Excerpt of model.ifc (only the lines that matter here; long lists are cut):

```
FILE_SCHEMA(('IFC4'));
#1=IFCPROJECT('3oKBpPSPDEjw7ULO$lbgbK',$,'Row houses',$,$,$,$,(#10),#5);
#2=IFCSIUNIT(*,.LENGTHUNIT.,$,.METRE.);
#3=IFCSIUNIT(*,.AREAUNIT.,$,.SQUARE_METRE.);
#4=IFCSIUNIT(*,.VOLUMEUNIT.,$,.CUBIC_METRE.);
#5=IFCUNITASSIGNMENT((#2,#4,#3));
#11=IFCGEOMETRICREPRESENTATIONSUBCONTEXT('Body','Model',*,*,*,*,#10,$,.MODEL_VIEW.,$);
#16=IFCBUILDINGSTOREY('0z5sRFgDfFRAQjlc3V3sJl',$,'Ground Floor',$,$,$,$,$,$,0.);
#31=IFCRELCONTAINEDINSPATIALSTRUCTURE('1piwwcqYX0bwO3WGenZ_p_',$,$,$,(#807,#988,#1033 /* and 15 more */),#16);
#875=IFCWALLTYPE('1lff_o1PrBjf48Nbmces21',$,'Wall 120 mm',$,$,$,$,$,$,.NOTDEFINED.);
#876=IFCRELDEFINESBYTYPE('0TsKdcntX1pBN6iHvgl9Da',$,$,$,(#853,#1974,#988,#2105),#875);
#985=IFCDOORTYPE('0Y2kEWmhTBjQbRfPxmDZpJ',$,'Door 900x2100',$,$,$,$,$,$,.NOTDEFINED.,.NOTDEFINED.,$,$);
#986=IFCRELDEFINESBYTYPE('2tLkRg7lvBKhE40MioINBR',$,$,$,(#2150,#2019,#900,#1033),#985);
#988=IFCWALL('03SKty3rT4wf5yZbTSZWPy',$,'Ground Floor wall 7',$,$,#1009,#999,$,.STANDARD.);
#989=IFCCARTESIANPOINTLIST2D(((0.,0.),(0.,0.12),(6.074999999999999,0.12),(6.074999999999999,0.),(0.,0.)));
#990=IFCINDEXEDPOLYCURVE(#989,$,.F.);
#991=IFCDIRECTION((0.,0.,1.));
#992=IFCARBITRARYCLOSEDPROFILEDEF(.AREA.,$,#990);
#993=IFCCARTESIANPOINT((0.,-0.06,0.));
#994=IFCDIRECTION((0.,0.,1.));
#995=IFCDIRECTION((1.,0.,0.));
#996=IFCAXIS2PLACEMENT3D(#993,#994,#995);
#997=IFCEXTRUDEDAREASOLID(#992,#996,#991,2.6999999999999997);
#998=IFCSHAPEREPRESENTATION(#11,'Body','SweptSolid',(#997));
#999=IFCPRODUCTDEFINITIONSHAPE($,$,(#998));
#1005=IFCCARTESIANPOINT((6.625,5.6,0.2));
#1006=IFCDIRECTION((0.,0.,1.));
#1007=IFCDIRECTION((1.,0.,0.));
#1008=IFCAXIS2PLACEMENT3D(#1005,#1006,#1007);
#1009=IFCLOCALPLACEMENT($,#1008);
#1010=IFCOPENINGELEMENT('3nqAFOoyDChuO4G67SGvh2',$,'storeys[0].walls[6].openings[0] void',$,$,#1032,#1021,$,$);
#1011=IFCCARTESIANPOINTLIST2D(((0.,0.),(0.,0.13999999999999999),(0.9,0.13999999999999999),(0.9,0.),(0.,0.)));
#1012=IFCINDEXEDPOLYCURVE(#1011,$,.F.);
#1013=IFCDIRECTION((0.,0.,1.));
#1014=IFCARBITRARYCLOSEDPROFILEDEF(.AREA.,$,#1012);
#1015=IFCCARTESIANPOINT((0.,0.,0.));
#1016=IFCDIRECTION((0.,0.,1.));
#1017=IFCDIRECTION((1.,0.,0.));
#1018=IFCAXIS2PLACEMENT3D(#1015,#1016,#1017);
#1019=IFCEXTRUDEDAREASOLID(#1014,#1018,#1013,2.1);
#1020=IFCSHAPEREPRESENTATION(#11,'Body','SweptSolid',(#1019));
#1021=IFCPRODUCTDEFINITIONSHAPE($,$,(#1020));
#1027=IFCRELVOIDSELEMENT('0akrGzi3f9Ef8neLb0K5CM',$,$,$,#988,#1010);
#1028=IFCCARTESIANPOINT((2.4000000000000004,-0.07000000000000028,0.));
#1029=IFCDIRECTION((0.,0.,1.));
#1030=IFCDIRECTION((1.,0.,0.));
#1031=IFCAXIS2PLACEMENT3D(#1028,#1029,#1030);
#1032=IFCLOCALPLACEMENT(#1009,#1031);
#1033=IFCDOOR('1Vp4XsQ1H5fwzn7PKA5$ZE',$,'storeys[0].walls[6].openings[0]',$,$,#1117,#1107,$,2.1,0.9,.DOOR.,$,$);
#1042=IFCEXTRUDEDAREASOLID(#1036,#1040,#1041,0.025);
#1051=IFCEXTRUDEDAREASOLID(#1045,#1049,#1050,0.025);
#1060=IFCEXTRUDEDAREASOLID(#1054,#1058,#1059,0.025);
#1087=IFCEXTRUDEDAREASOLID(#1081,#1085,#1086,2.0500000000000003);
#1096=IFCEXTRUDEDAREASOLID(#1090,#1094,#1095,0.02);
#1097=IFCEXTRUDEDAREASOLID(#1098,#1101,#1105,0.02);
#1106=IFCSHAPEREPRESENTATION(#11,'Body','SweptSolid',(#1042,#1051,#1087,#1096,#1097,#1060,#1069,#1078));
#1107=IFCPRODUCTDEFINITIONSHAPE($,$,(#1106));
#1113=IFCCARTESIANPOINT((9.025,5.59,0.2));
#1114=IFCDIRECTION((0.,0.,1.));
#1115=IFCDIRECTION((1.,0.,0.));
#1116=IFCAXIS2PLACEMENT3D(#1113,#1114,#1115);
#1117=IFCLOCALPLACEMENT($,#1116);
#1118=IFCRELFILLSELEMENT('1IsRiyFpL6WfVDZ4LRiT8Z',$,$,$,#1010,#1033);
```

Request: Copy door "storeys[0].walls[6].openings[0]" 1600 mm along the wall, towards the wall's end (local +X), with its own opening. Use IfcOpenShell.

```python
import ifcopenshell
import ifcopenshell.api.feature
import ifcopenshell.api.geometry
import ifcopenshell.api.root
import ifcopenshell.geom
import ifcopenshell.util.element
import ifcopenshell.util.placement
import ifcopenshell.util.shape
import ifcopenshell.util.unit

model = ifcopenshell.open("model.ifc")
unit_scale = ifcopenshell.util.unit.calculate_unit_scale(model)
settings = ifcopenshell.geom.settings()


def volume(element):
    """Net volume in cubic metres, openings subtracted."""
    shape = ifcopenshell.geom.create_shape(settings, element)
    return ifcopenshell.util.shape.get_volume(shape.geometry)


door = model.by_guid("1Vp4XsQ1H5fwzn7PKA5$ZE")
opening = door.FillsVoids[0].RelatingOpeningElement
wall = opening.VoidsElements[0].RelatingBuildingElement
before = volume(wall)
shift = ifcopenshell.util.placement.get_local_placement(wall.ObjectPlacement)[:3, 0] * 1.6 / unit_scale

# copy_class copies the void relationship, type, container and properties, but no geometry.
new_opening = ifcopenshell.api.root.copy_class(model, product=opening)
new_opening.Representation = ifcopenshell.util.element.copy_deep(
    model, opening.Representation, exclude=["IfcGeometricRepresentationContext", "IfcRepresentationMap"]
)
new_door = ifcopenshell.api.root.copy_class(model, product=door)
new_door.Representation = ifcopenshell.util.element.copy_deep(
    model, door.Representation, exclude=["IfcGeometricRepresentationContext", "IfcRepresentationMap"]
)
ifcopenshell.api.feature.add_filling(model, opening=new_opening, element=new_door)

for old, new in ((opening, new_opening), (door, new_door)):
    matrix = ifcopenshell.util.placement.get_local_placement(old.ObjectPlacement)
    matrix[:3, 3] += shift
    ifcopenshell.api.geometry.edit_object_placement(model, product=new, matrix=matrix, is_si=False)

after = volume(wall)

print(f"wall volume {before:.3f} -> {after:.3f} m3")

model.write("model_updated.ifc")
```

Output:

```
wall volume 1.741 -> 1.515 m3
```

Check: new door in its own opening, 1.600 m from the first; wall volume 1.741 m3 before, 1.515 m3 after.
